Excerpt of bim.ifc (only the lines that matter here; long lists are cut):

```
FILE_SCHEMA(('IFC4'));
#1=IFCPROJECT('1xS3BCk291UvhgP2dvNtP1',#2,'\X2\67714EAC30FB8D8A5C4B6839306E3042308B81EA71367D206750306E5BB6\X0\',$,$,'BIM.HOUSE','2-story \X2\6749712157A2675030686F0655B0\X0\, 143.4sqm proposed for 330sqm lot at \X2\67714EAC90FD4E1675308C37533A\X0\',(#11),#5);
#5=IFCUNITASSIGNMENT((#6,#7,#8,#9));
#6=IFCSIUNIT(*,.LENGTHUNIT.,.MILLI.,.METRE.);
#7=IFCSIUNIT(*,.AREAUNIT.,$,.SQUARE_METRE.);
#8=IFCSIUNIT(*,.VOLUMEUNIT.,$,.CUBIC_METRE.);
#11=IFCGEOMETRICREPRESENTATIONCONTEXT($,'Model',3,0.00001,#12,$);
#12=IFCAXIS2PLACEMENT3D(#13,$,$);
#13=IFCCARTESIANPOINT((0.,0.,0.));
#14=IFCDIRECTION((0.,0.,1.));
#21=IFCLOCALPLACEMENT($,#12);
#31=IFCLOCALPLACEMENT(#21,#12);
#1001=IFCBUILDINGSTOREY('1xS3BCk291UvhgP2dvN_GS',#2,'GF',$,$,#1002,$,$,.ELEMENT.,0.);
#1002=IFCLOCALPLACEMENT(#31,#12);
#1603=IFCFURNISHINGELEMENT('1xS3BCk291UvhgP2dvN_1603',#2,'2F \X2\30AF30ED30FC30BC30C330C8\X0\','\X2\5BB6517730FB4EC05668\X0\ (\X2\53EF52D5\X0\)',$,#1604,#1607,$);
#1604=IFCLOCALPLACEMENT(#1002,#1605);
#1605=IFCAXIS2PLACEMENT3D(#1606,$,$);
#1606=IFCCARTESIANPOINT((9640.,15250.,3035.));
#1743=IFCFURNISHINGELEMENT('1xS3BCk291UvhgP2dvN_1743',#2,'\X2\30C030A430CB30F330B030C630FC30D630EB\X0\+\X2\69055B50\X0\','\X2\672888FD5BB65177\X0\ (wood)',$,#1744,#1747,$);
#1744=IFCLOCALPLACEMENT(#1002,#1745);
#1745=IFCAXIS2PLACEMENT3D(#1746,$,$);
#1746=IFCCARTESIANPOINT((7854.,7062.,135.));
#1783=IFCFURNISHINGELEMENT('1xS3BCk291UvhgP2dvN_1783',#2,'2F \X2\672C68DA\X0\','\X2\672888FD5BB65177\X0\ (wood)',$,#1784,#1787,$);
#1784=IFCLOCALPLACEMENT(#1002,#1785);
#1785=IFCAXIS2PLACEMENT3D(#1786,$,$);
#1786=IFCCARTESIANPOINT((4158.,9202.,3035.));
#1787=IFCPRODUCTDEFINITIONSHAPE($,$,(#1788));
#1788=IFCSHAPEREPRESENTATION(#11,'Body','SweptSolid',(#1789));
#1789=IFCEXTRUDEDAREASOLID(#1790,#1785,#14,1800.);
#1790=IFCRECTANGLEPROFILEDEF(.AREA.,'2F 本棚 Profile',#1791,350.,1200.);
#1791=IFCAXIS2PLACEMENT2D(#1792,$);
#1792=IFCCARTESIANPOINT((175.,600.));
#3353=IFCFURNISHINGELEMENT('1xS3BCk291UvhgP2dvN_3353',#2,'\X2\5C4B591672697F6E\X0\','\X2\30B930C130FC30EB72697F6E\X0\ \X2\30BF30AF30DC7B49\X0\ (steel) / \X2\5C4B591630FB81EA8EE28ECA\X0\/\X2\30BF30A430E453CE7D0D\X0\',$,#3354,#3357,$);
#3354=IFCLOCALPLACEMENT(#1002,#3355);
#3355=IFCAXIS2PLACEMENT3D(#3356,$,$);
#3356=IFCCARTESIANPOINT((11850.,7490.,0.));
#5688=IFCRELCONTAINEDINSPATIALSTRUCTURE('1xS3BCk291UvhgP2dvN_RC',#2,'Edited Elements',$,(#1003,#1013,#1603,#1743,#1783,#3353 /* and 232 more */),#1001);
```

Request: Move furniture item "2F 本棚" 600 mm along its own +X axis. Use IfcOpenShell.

```python
import ifcopenshell
import ifcopenshell.api.geometry
import ifcopenshell.util.placement
import ifcopenshell.util.unit

model = ifcopenshell.open("bim.ifc")
unit_scale = ifcopenshell.util.unit.calculate_unit_scale(model)

item = model.by_guid("1xS3BCk291UvhgP2dvN_1783")
matrix = ifcopenshell.util.placement.get_local_placement(item.ObjectPlacement)
matrix[:3, 3] += matrix[:3, 0] * 0.6 / unit_scale
ifcopenshell.api.geometry.edit_object_placement(model, product=item, matrix=matrix, is_si=False)

print(ifcopenshell.util.placement.get_local_placement(item.ObjectPlacement).round(3) + 0.0)

model.write("bim-out.ifc")
```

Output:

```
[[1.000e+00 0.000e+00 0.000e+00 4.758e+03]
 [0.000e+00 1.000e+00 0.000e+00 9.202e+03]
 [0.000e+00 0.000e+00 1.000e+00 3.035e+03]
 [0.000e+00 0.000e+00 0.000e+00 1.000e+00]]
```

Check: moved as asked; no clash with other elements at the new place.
